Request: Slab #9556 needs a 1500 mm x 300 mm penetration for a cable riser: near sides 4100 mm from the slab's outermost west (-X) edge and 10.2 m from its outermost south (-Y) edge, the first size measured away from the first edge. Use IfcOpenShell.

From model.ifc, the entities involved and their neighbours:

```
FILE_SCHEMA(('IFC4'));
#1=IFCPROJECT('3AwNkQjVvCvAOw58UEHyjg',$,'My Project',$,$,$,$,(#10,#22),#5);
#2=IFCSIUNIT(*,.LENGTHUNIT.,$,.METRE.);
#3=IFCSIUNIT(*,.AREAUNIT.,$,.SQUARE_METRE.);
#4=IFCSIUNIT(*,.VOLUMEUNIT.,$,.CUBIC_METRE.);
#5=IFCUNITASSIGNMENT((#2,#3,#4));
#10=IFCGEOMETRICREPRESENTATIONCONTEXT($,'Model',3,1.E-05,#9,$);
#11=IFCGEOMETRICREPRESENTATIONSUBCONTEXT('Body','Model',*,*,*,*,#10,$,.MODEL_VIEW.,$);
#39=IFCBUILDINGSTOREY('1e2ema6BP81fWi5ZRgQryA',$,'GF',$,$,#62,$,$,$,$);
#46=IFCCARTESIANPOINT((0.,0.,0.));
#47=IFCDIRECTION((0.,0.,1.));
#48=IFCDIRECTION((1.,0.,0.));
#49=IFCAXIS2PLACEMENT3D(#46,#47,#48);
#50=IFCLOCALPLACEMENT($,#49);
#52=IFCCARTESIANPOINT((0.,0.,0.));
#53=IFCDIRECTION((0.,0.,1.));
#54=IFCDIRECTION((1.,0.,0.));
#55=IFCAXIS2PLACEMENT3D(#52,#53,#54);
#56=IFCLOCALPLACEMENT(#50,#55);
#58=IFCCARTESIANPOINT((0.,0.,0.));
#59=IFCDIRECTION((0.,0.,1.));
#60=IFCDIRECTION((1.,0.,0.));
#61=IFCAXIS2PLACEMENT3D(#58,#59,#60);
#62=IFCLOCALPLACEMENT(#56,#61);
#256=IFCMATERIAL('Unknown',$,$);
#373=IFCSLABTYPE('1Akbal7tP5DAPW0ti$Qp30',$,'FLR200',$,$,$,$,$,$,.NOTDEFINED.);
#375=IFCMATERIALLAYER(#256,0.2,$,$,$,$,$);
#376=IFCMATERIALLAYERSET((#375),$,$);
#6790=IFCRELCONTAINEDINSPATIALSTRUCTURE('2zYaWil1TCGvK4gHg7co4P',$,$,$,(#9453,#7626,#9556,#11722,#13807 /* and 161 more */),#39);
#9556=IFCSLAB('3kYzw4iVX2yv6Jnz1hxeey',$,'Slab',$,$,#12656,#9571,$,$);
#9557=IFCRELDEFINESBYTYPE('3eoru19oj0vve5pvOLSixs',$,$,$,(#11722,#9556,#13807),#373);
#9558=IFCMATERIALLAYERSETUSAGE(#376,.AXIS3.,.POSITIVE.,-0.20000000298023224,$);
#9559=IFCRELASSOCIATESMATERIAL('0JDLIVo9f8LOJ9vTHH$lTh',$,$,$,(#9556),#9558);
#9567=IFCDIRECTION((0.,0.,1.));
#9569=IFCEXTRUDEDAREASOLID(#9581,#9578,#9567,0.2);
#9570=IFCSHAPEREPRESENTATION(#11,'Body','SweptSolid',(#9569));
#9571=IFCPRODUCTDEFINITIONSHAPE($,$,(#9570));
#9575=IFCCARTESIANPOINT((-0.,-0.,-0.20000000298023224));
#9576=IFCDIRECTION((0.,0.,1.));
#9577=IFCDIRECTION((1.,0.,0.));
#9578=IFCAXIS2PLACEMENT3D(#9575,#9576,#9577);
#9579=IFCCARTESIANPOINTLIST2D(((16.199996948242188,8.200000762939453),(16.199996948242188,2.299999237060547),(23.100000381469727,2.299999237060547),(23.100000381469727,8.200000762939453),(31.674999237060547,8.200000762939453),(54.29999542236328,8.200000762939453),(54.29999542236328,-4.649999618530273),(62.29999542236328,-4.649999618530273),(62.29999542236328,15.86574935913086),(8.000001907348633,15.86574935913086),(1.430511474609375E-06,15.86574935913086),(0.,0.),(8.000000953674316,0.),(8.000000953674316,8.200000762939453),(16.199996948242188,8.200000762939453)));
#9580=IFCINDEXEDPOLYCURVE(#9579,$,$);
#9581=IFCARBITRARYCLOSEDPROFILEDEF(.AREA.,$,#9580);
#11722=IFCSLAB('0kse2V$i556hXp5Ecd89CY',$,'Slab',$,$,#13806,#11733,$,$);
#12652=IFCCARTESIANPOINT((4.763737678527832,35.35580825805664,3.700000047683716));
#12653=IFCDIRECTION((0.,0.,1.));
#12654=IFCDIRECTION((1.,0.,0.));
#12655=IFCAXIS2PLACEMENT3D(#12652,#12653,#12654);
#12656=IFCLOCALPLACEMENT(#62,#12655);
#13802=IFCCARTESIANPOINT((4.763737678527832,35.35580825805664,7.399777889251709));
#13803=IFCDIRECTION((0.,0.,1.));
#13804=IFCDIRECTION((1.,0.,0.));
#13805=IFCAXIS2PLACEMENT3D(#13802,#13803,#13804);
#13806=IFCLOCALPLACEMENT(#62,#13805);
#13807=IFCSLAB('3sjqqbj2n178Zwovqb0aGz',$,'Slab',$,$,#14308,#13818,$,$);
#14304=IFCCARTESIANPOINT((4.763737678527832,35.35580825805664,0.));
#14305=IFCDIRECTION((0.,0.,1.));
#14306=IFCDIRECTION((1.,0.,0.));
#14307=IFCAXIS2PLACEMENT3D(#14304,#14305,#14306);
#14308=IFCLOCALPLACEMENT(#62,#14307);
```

```python
import numpy as np
import ifcopenshell
import ifcopenshell.api.feature
import ifcopenshell.api.geometry
import ifcopenshell.api.root
import ifcopenshell.geom
import ifcopenshell.util.placement
import ifcopenshell.util.representation
import ifcopenshell.util.shape
import ifcopenshell.util.unit

model = ifcopenshell.open("model.ifc")
unit_scale = ifcopenshell.util.unit.calculate_unit_scale(model)
settings = ifcopenshell.geom.settings()


def volume(element):
    """Net volume in cubic metres, openings subtracted."""
    shape = ifcopenshell.geom.create_shape(settings, element)
    return ifcopenshell.util.shape.get_volume(shape.geometry)


slab = model.by_guid("3kYzw4iVX2yv6Jnz1hxeey")
before = volume(slab)

# Extent in the slab's own axes, in metres. The edges named are its -X and -Y sides.
slab_shape = ifcopenshell.geom.create_shape(settings, slab)
vertices = ifcopenshell.util.shape.get_vertices(slab_shape.geometry)
x_min, y_min, bottom = vertices.min(axis=0)
top = vertices[:, 2].max()

opening = ifcopenshell.api.root.create_entity(model, ifc_class="IfcOpeningElement", name="Cable riser opening", predefined_type="OPENING")
context = ifcopenshell.util.representation.get_context(model, "Model", "Body", "MODEL_VIEW")
width, depth = 1.5, 0.3
outline = [(0.0, 0.0), (width, 0.0), (width, depth), (0.0, depth), (0.0, 0.0)]
# Overshoot both faces by 50 mm so the cut is clean.
shape = ifcopenshell.api.geometry.add_slab_representation(
    model, context=context, depth=top - bottom + 0.1, polyline=outline
)
ifcopenshell.api.geometry.assign_representation(model, product=opening, representation=shape)

matrix = ifcopenshell.util.placement.get_local_placement(slab.ObjectPlacement)
matrix[:, 3] = matrix @ np.append(np.array([x_min + 4.1, y_min + 10.2, bottom - 0.05]) / unit_scale, 1.0)
ifcopenshell.api.geometry.edit_object_placement(model, product=opening, matrix=matrix, is_si=False)
ifcopenshell.api.feature.add_feature(model, feature=opening, element=slab)

after = volume(slab)

print(f"slab volume {before:.3f} -> {after:.3f} m3")

model.write("model-out.ifc")
```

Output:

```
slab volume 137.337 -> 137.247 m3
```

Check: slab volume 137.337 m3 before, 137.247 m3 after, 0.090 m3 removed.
